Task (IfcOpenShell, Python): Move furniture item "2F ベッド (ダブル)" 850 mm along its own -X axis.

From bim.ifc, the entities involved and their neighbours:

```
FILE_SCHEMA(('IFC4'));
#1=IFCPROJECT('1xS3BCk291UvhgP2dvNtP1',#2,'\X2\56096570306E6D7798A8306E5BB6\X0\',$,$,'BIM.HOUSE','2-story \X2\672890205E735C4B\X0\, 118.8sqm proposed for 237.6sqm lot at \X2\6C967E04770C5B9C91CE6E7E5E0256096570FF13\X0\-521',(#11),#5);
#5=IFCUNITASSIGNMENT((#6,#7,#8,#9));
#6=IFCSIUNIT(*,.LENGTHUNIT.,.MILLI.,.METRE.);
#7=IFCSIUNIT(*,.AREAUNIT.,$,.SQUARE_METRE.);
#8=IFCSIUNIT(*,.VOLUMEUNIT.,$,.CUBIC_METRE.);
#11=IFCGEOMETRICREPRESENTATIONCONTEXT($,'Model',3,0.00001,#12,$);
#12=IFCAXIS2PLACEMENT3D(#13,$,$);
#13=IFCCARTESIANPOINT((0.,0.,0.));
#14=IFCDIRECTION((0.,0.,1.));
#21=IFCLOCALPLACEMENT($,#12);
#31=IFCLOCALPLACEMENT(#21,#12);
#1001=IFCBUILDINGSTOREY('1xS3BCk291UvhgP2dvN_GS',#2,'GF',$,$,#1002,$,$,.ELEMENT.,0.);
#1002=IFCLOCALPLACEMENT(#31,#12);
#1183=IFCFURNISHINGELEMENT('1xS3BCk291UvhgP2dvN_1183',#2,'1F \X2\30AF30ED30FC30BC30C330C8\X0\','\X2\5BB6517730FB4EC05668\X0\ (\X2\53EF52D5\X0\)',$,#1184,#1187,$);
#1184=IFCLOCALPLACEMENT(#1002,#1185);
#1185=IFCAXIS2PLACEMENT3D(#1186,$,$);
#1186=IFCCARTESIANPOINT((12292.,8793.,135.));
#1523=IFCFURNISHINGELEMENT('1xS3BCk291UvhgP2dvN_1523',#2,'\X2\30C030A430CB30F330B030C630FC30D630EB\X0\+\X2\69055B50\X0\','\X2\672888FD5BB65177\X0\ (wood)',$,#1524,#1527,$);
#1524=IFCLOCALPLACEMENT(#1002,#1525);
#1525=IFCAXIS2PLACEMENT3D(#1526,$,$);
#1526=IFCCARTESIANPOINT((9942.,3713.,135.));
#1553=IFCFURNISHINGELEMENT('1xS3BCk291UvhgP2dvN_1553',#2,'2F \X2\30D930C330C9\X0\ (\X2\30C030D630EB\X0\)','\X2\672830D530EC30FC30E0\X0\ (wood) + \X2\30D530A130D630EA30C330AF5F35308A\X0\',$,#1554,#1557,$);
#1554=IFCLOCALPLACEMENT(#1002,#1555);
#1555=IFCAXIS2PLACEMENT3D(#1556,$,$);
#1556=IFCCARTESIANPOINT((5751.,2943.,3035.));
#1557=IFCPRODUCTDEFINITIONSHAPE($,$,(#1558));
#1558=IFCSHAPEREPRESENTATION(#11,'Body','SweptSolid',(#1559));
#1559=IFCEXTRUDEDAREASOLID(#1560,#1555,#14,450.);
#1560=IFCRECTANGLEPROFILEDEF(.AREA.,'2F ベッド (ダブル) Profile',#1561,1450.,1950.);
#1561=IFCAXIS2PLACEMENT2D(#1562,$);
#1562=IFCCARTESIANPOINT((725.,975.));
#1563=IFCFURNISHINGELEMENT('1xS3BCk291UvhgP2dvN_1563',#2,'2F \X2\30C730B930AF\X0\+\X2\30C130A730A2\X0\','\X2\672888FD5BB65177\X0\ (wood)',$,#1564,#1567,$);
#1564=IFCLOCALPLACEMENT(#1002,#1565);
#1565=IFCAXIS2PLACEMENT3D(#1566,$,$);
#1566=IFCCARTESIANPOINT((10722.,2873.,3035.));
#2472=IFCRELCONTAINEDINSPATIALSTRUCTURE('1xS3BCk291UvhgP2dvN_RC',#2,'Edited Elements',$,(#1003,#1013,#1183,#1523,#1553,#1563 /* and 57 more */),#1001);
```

```python
import ifcopenshell
import ifcopenshell.api.geometry
import ifcopenshell.util.placement
import ifcopenshell.util.unit

model = ifcopenshell.open("bim.ifc")
unit_scale = ifcopenshell.util.unit.calculate_unit_scale(model)

item = model.by_guid("1xS3BCk291UvhgP2dvN_1553")
matrix = ifcopenshell.util.placement.get_local_placement(item.ObjectPlacement)
matrix[:3, 3] -= matrix[:3, 0] * 0.85 / unit_scale
ifcopenshell.api.geometry.edit_object_placement(model, product=item, matrix=matrix, is_si=False)

print(ifcopenshell.util.placement.get_local_placement(item.ObjectPlacement).round(3) + 0.0)

model.write("bim-out.ifc")
```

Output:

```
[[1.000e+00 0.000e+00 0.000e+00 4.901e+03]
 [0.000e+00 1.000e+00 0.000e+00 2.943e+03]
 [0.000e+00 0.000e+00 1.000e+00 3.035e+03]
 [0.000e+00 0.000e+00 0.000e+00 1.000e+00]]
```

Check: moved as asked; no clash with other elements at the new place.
